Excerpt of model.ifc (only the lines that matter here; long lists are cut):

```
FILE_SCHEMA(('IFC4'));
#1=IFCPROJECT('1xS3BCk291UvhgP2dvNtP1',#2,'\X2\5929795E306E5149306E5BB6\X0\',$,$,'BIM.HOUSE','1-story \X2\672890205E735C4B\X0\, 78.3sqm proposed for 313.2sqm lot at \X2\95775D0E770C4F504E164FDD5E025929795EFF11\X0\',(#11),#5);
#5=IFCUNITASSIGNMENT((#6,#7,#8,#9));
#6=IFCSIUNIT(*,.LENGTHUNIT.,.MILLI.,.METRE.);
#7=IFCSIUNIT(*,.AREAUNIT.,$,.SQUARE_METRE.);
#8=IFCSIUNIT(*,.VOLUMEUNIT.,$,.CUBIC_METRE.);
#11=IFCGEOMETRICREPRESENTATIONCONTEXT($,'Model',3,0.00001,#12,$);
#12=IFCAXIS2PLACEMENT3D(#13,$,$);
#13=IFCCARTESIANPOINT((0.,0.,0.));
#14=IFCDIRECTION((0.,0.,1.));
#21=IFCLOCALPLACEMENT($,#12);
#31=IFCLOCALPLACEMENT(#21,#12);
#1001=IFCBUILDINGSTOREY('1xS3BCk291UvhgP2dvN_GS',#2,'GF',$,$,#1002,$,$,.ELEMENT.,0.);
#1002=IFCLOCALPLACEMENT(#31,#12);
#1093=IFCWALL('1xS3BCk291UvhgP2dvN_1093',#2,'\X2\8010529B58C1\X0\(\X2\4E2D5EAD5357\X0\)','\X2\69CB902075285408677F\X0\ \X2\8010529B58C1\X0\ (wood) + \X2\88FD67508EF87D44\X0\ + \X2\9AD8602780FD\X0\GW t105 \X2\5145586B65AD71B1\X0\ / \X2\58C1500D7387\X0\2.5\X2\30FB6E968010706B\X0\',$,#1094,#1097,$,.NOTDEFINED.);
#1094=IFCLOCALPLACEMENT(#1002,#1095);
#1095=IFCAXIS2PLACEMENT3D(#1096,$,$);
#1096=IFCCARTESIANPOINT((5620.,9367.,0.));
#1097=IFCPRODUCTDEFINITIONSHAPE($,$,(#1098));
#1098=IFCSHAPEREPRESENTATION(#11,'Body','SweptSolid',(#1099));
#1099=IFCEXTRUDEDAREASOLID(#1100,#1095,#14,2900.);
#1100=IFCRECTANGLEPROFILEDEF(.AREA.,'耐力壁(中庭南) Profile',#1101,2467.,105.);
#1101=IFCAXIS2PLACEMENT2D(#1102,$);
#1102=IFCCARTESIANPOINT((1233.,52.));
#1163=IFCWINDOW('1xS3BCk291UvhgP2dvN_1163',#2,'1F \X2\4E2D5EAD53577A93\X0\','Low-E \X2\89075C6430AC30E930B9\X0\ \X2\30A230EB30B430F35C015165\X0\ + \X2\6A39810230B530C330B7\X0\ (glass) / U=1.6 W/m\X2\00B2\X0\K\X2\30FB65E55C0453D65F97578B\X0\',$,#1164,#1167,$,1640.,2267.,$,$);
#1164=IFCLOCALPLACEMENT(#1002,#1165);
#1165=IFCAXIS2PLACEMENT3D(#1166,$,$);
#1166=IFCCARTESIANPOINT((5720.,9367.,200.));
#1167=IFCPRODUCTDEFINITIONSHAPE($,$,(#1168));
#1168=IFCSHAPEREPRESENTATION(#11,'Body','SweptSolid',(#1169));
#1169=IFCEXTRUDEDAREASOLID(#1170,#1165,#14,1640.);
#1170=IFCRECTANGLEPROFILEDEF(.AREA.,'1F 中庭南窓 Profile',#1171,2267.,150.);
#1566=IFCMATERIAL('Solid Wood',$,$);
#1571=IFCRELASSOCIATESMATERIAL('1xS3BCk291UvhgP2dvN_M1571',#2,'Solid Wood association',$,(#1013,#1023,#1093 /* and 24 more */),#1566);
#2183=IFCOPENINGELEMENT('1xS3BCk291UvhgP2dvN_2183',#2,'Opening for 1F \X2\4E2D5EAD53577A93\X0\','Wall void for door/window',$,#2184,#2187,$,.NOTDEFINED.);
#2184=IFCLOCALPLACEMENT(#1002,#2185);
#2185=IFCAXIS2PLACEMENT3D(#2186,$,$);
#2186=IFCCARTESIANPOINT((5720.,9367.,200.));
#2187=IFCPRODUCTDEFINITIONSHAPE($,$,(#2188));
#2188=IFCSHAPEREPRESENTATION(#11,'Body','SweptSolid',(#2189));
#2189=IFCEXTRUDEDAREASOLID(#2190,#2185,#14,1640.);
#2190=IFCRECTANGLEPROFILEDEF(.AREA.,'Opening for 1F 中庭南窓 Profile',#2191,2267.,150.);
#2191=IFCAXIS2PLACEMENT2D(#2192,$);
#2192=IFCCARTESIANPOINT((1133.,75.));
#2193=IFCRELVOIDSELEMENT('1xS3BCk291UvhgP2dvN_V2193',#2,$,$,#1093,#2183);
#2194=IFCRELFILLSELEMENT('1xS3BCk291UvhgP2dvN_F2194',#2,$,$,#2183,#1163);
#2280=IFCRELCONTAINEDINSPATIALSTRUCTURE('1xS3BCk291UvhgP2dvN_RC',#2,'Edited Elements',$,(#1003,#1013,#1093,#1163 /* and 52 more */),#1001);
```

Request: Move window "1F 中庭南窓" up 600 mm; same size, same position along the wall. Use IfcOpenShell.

```python
import numpy as np
import ifcopenshell
import ifcopenshell.api.geometry
import ifcopenshell.util.placement
import ifcopenshell.util.unit

model = ifcopenshell.open("model.ifc")
unit_scale = ifcopenshell.util.unit.calculate_unit_scale(model)

window = model.by_guid("1xS3BCk291UvhgP2dvN_1163")
opening = window.FillsVoids[0].RelatingOpeningElement
dz = 0.6 / unit_scale

shift = np.array([0.0, 0.0, dz])
# The window is not placed relative to its opening, so move both.
for product in (opening, window):
    matrix = ifcopenshell.util.placement.get_local_placement(product.ObjectPlacement)
    matrix[:3, 3] += shift
    ifcopenshell.api.geometry.edit_object_placement(model, product=product, matrix=matrix, is_si=False)

print(f"moved by {dz * unit_scale:+.3f} m")

model.write("model_updated.ifc")
```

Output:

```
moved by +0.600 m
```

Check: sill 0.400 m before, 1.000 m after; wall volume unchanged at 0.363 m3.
